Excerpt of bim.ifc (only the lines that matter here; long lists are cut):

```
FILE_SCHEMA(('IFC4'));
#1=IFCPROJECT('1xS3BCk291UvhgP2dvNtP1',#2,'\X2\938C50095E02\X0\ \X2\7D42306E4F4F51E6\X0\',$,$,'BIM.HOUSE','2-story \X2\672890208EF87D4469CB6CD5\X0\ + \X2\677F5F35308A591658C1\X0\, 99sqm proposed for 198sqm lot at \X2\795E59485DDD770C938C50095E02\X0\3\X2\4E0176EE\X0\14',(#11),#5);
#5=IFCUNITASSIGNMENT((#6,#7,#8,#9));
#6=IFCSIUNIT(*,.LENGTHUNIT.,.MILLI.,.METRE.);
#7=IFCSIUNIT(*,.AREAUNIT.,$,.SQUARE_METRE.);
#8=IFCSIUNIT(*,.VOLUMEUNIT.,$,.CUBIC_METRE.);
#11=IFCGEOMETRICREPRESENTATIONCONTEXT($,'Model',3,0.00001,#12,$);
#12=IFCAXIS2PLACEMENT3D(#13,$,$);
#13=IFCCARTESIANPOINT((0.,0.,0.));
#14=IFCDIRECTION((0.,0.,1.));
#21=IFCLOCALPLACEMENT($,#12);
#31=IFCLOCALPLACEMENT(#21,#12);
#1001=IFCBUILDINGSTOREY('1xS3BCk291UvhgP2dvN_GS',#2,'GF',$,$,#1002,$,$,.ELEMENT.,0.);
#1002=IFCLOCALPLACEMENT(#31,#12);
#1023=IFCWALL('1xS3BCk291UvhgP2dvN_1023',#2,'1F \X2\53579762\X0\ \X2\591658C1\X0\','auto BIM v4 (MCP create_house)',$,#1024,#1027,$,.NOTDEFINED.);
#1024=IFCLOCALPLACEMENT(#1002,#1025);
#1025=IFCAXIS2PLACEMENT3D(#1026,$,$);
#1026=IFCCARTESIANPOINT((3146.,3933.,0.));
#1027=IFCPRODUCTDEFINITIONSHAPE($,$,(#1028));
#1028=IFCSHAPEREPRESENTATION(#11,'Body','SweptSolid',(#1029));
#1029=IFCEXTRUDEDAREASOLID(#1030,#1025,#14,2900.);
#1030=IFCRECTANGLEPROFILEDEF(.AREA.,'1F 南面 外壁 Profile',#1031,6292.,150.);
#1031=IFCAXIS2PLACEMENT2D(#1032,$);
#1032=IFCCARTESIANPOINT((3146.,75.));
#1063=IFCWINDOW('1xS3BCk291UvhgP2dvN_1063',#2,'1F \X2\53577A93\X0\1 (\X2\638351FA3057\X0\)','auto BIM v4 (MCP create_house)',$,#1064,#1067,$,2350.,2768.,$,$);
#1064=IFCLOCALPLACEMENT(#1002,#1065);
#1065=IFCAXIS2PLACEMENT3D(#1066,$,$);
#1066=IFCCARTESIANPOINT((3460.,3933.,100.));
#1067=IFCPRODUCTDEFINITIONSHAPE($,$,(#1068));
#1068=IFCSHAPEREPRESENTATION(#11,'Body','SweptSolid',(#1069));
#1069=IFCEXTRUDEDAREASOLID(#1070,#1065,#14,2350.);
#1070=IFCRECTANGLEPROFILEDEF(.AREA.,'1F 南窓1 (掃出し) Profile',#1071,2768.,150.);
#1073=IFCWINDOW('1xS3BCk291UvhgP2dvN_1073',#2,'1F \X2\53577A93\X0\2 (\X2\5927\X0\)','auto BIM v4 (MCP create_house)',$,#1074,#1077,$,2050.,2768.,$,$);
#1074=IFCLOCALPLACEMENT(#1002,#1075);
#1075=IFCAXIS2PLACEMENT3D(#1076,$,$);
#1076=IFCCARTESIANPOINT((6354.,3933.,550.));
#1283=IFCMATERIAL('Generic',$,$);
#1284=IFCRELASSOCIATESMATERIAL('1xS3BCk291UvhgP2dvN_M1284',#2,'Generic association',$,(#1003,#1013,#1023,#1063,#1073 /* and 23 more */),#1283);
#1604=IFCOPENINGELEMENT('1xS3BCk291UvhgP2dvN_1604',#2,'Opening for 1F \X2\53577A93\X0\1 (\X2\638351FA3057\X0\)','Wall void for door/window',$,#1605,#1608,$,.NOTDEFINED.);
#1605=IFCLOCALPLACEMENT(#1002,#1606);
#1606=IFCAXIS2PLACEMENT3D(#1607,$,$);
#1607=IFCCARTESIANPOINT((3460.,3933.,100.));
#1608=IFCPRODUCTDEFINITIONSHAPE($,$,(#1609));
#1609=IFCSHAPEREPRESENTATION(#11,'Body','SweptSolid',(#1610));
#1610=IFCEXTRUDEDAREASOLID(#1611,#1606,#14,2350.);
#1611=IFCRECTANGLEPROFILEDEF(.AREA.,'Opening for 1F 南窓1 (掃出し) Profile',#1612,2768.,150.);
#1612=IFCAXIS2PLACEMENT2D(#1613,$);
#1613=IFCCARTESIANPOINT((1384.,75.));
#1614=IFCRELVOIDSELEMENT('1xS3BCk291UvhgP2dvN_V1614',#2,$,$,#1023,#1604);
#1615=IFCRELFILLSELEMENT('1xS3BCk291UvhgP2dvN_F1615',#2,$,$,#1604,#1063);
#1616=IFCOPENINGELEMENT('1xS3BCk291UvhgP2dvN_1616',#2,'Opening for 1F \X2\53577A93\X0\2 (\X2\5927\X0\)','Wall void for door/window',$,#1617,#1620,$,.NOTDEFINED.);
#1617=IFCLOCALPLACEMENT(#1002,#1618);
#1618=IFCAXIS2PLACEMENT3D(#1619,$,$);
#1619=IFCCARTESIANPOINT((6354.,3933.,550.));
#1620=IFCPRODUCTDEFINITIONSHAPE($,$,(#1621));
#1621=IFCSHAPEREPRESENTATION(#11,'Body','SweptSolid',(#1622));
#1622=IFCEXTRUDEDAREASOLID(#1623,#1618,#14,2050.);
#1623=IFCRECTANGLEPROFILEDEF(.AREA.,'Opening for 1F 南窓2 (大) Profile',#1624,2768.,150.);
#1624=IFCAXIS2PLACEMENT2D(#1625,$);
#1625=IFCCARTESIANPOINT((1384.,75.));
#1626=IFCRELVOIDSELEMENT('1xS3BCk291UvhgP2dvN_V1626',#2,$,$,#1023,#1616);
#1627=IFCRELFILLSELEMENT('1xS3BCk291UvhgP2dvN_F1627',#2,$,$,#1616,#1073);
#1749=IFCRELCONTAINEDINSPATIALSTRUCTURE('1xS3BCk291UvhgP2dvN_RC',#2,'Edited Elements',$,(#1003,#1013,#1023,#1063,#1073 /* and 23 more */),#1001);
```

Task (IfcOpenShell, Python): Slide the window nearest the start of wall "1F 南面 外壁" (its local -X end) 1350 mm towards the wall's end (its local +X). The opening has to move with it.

```python
import ifcopenshell
import ifcopenshell.api.geometry
import ifcopenshell.util.placement

model = ifcopenshell.open("bim.ifc")

window = model.by_guid("1xS3BCk291UvhgP2dvN_1063")
opening = window.FillsVoids[0].RelatingOpeningElement
wall = opening.VoidsElements[0].RelatingBuildingElement

wall_matrix = ifcopenshell.util.placement.get_local_placement(wall.ObjectPlacement)
shift = wall_matrix[:3, 0] * 1350.0
before = ifcopenshell.util.placement.get_local_placement(window.ObjectPlacement)[:3, 3].copy()

# The window is not placed relative to its opening, so move both.
for product in (opening, window):
    matrix = ifcopenshell.util.placement.get_local_placement(product.ObjectPlacement)
    matrix[:3, 3] += shift
    ifcopenshell.api.geometry.edit_object_placement(model, product=product, matrix=matrix, is_si=False)

after = ifcopenshell.util.placement.get_local_placement(window.ObjectPlacement)[:3, 3]
print("window moved by", (after - before).round(3) + 0.0)

model.write("bim_rev.ifc")
```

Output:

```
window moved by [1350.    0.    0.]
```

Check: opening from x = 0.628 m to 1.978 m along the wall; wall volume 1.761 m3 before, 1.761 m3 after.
